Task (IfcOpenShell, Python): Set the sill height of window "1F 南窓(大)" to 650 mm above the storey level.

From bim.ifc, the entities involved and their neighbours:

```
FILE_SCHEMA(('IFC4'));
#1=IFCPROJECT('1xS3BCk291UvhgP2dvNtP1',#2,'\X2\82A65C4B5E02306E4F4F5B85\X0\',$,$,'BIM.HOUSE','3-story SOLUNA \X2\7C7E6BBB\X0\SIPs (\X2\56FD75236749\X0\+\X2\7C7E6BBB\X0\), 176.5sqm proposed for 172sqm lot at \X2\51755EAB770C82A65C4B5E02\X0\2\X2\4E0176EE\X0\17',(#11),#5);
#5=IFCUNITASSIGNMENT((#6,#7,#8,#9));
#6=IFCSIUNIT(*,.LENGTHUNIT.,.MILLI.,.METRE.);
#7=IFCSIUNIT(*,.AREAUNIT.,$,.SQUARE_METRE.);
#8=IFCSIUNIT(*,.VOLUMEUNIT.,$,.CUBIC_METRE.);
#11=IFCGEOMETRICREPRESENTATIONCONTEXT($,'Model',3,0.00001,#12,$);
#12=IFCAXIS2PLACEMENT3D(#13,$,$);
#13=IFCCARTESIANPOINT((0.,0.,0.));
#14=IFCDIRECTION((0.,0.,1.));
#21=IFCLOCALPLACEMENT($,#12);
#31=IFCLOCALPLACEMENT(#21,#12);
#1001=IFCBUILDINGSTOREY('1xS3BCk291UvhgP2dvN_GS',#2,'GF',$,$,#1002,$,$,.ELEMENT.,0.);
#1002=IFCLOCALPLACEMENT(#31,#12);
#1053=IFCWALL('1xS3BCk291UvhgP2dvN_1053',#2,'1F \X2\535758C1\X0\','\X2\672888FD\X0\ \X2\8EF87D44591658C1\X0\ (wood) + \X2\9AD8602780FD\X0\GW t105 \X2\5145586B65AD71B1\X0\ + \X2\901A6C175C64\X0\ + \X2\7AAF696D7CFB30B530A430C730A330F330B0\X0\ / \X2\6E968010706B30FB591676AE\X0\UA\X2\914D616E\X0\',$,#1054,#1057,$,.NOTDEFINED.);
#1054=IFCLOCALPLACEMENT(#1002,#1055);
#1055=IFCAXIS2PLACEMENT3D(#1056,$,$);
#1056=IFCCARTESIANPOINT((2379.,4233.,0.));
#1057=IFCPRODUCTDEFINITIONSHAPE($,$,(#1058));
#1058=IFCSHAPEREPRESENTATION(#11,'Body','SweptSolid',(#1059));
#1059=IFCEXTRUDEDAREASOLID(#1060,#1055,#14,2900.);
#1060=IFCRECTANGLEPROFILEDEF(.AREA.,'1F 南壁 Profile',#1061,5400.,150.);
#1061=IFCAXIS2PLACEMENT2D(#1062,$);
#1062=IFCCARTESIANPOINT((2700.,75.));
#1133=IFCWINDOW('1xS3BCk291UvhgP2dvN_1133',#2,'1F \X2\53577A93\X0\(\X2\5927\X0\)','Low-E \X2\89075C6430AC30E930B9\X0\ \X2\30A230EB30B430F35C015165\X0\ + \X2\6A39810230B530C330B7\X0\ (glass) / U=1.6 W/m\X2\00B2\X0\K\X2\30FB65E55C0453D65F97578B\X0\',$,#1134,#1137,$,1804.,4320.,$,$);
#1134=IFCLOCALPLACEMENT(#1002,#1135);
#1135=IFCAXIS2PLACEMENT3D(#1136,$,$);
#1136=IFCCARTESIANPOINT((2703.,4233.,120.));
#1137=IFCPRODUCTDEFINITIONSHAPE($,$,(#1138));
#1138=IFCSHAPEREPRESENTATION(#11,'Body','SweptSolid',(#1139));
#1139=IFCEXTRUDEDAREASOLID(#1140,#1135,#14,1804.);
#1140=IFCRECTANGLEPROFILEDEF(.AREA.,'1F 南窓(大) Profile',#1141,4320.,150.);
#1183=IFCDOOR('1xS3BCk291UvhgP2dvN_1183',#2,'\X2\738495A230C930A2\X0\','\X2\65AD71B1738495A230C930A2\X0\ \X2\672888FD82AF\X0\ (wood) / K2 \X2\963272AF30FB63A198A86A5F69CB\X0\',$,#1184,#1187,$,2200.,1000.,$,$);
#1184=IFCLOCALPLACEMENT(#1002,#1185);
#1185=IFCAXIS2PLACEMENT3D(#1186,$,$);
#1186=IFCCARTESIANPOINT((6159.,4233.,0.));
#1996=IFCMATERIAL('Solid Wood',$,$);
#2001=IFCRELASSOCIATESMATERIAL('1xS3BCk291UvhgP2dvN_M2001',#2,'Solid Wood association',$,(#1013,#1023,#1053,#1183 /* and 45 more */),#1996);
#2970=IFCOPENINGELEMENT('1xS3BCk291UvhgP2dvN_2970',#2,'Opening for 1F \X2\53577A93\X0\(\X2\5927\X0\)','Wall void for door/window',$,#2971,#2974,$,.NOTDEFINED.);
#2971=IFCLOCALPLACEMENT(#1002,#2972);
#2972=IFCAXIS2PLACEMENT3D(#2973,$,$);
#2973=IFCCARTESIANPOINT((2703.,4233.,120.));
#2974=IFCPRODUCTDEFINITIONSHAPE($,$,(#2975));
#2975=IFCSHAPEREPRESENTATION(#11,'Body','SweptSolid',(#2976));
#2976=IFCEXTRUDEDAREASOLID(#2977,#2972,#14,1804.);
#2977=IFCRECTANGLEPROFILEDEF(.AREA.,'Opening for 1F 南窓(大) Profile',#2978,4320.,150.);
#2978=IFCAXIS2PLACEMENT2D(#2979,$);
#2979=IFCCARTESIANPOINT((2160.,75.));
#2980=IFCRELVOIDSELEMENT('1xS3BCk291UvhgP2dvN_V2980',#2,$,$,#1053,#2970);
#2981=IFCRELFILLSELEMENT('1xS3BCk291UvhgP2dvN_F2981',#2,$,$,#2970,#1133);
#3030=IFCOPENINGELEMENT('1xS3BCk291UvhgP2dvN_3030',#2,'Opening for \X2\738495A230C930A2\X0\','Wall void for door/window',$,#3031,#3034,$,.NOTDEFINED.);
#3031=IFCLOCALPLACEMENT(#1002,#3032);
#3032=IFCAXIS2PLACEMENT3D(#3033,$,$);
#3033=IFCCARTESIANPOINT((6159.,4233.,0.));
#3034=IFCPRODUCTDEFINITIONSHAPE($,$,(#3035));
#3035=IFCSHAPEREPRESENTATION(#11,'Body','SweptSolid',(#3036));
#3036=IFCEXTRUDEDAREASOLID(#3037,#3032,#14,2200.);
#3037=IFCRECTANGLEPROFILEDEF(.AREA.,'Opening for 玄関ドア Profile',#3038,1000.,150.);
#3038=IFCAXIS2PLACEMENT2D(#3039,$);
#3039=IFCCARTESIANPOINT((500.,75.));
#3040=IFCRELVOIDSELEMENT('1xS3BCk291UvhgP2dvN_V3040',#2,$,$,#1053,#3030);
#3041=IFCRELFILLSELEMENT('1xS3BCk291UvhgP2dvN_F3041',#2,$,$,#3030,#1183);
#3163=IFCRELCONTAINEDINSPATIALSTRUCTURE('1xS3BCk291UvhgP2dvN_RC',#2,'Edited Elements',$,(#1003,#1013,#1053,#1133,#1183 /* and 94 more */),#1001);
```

```python
import numpy as np
import ifcopenshell
import ifcopenshell.api.geometry
import ifcopenshell.geom
import ifcopenshell.util.element
import ifcopenshell.util.placement
import ifcopenshell.util.shape
import ifcopenshell.util.unit

model = ifcopenshell.open("bim.ifc")
unit_scale = ifcopenshell.util.unit.calculate_unit_scale(model)

window = model.by_guid("1xS3BCk291UvhgP2dvN_1133")
opening = window.FillsVoids[0].RelatingOpeningElement
storey = ifcopenshell.util.element.get_container(window, ifc_class="IfcBuildingStorey")
level = ifcopenshell.util.placement.get_local_placement(storey.ObjectPlacement)[2, 3]

# The opening's origin need not be at the sill, so measure its lowest point.
shape = ifcopenshell.geom.create_shape(ifcopenshell.geom.settings(), opening)
bottom = ifcopenshell.util.shape.get_shape_bottom_elevation(shape, shape.geometry) / unit_scale
dz = level + 0.65 / unit_scale - bottom

shift = np.array([0.0, 0.0, dz])
# The window is not placed relative to its opening, so move both.
for product in (opening, window):
    matrix = ifcopenshell.util.placement.get_local_placement(product.ObjectPlacement)
    matrix[:3, 3] += shift
    ifcopenshell.api.geometry.edit_object_placement(model, product=product, matrix=matrix, is_si=False)

print(f"moved by {dz * unit_scale:+.3f} m")

model.write("bim_edited.ifc")
```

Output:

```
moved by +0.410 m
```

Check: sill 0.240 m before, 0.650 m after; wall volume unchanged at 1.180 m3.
